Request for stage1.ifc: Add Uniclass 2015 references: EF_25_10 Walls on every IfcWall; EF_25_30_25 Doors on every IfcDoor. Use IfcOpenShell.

First a look at what the model holds.

```python
import ifcopenshell

model = ifcopenshell.open("stage1.ifc")
print(model.schema)
print("classifications:", [c.Name for c in model.by_type("IfcClassification")])
for ifc_class in ("IfcDoor", "IfcRoof", "IfcStair", "IfcWall", "IfcWindow"):
    print(ifc_class, len(model.by_type(ifc_class)))
```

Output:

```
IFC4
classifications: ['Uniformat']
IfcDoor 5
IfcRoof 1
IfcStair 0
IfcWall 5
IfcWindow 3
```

```python
import ifcopenshell
import ifcopenshell.api.classification

model = ifcopenshell.open("stage1.ifc")

system = ifcopenshell.api.classification.add_classification(model, classification="Uniclass 2015")

codes = {
    "IfcWall": ("EF_25_10", "Walls"),
    "IfcDoor": ("EF_25_30_25", "Doors"),
}
for ifc_class, (code, name) in codes.items():
    products = model.by_type(ifc_class)
    ifcopenshell.api.classification.add_reference(
        model, products=products, classification=system, identification=code, name=name
    )
    print(code, len(products))

model.write("stage1_updated.ifc")
```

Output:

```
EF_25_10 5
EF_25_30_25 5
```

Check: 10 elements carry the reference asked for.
